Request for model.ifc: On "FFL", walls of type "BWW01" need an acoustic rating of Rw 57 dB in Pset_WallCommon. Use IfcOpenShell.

First a look at what the model holds.

```python
import ifcopenshell
import ifcopenshell.util.element

model = ifcopenshell.open("model.ifc")
print(model.schema)
storey = next(s for s in model.by_type("IfcBuildingStorey") if s.Name == "FFL")
walls = [e for e in ifcopenshell.util.element.get_decomposition(storey) if e.is_a("IfcWall")]
seen = {}
for e in walls:
    element_type = ifcopenshell.util.element.get_type(e)
    key = (element_type.Name if element_type != e and element_type else None, ifcopenshell.util.element.get_pset(e, "Pset_WallCommon", "AcousticRating"))
    seen[key] = seen.get(key, 0) + 1
for (name, value), count in sorted(seen.items(), key=str):
    print(count, "x", name, "|", value)
```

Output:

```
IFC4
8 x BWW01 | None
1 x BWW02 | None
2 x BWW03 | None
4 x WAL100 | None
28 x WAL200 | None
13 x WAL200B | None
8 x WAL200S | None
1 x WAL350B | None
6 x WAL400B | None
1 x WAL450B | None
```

```python
import ifcopenshell
import ifcopenshell.api.pset
import ifcopenshell.util.element

model = ifcopenshell.open("model.ifc")

storey = next(s for s in model.by_type("IfcBuildingStorey") if s.Name == "FFL")
walls = [e for e in ifcopenshell.util.element.get_decomposition(storey) if e.is_a("IfcWall")]

count = 0
for e in walls:
    element_type = ifcopenshell.util.element.get_type(e)
    if element_type in (None, e) or element_type.Name != "BWW01":
        continue
    # add_pset returns the element's existing set when there is one.
    pset = ifcopenshell.api.pset.add_pset(model, product=e, name="Pset_WallCommon")
    ifcopenshell.api.pset.edit_pset(model, pset=pset, properties={"AcousticRating": "Rw 57 dB"})
    count += 1

print(count, "walls updated")

model.write("model-out.ifc")
```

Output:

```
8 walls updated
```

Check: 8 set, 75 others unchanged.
